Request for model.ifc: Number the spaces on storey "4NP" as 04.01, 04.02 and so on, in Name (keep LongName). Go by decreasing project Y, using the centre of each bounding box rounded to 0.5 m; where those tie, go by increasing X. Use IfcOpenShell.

First a look at what the model holds.

```python
import ifcopenshell
import ifcopenshell.util.element
import ifcopenshell.util.placement

model = ifcopenshell.open("model.ifc")
print(model.schema)
storey = next(s for s in model.by_type("IfcBuildingStorey") if s.Name == "4NP")
spaces = [e for e in ifcopenshell.util.element.get_decomposition(storey) if e.is_a("IfcSpace")]
for e in sorted(spaces, key=lambda e: e.id()):
    origin = ifcopenshell.util.placement.get_local_placement(e.ObjectPlacement)[:3, 3]
    print(e.id(), e.Name, e.LongName, origin.round(2) + 0.0, sep=" | ")
```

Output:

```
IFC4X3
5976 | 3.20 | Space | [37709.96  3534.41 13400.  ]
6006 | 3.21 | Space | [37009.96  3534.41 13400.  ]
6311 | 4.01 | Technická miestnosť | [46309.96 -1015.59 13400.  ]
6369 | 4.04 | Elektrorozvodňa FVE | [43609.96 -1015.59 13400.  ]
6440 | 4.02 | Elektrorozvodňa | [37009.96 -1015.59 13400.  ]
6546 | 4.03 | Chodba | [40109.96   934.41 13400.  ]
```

```python
import ifcopenshell
import ifcopenshell.geom
import ifcopenshell.util.element
import ifcopenshell.util.shape

model = ifcopenshell.open("model.ifc")
settings = ifcopenshell.geom.settings()
settings.set("use-world-coords", True)


def centre(element):
    shape = ifcopenshell.geom.create_shape(settings, element)
    return ifcopenshell.util.shape.get_bbox_centroid(shape.geometry)


storey = next(s for s in model.by_type("IfcBuildingStorey") if s.Name == "4NP")
spaces = [e for e in ifcopenshell.util.element.get_decomposition(storey) if e.is_a("IfcSpace")]

# Insertion points can sit at a corner or the storey origin, so sort by the geometry (in metres).
centres = {e: centre(e) for e in spaces}
spaces.sort(key=lambda e: (-round(centres[e][1] / 0.5), centres[e][0]))

for i, e in enumerate(spaces, start=1):
    number = f"04.{i:02d}"
    e.Name = number
    print(e.id(), number)

model.write("model-out.ifc")
```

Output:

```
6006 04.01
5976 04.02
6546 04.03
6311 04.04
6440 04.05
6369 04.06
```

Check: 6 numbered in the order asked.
